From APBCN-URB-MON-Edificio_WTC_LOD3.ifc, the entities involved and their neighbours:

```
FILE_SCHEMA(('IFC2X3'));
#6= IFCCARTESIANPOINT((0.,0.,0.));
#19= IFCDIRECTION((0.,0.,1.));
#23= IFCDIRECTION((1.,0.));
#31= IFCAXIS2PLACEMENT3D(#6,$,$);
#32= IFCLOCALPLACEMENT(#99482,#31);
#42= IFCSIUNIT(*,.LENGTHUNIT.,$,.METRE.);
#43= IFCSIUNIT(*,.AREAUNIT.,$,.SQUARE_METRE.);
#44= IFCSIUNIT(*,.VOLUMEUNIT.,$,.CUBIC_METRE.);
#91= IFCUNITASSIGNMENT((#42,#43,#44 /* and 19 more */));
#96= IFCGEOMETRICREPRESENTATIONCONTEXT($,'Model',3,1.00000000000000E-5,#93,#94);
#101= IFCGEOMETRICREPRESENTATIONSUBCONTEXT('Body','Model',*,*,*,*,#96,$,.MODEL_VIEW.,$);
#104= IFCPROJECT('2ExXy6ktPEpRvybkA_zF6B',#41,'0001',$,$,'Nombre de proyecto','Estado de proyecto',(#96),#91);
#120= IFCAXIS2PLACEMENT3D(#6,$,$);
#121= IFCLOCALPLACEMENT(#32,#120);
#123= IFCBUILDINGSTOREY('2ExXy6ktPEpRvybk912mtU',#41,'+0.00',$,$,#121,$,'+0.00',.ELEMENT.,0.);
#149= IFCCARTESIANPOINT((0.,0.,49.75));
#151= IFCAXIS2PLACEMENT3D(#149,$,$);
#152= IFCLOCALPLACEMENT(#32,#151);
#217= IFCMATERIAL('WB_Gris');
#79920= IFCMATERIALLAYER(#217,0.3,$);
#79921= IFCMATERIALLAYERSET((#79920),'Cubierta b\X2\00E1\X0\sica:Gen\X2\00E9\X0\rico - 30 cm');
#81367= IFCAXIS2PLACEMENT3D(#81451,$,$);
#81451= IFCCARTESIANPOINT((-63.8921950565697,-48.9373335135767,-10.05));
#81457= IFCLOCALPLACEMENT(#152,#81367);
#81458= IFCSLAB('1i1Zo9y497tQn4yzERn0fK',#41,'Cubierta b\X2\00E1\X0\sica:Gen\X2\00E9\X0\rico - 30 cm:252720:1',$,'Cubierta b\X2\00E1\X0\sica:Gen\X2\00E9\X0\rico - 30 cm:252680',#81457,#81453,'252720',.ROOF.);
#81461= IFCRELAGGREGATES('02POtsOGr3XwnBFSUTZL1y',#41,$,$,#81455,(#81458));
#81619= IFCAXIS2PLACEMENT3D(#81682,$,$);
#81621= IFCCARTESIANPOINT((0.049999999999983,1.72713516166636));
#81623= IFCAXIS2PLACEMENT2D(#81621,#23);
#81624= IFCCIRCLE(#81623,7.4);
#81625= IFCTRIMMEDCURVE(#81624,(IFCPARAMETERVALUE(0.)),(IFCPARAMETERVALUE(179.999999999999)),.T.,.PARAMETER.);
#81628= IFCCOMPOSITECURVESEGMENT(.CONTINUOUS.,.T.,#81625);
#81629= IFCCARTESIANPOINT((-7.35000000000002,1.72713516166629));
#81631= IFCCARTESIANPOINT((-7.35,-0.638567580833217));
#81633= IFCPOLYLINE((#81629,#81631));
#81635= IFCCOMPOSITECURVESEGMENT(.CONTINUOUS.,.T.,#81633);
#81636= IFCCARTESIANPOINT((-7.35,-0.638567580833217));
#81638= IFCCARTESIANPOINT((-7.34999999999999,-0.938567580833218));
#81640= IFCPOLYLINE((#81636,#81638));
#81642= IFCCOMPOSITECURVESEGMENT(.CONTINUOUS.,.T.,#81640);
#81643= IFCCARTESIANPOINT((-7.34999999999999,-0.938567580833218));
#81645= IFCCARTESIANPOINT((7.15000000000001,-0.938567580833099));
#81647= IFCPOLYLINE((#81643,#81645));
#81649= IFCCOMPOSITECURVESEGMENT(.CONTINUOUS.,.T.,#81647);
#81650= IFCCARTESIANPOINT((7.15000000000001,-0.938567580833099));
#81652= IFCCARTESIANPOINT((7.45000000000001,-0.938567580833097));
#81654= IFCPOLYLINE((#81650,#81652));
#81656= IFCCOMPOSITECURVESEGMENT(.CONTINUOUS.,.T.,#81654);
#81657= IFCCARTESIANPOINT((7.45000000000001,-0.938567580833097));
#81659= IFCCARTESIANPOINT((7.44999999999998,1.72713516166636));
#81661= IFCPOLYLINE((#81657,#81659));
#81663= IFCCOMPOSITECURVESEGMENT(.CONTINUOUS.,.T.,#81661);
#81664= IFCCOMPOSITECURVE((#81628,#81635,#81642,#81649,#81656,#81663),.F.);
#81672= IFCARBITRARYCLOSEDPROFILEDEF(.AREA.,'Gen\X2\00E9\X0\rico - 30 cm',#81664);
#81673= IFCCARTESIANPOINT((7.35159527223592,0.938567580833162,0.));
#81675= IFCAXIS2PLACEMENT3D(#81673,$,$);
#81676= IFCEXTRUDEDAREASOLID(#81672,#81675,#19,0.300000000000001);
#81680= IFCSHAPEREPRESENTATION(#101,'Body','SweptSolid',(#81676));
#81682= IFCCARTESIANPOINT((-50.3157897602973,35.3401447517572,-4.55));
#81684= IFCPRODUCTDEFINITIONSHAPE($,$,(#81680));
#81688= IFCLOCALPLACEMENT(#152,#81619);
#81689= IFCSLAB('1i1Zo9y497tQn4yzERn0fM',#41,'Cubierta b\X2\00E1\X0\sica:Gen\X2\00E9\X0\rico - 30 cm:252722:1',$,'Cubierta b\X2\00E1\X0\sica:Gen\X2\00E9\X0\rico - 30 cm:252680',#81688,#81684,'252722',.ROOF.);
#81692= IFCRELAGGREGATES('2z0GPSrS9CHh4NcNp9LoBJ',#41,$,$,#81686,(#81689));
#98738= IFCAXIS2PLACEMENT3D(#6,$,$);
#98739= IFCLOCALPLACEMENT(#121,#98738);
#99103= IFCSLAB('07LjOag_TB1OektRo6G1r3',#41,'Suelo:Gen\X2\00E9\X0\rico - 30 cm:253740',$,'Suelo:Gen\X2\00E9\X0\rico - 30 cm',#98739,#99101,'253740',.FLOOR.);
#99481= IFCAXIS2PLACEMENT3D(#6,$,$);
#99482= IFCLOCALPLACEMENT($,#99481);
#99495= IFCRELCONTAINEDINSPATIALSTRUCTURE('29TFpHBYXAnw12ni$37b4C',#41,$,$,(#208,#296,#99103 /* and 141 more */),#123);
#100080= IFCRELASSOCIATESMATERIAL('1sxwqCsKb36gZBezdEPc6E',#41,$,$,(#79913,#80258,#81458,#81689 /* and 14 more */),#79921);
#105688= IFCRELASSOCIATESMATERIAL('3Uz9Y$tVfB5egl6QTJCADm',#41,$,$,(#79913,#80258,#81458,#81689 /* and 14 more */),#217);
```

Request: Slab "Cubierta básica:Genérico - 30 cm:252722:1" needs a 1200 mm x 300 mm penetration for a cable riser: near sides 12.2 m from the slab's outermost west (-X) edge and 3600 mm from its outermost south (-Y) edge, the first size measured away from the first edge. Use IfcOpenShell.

```python
import numpy as np
import ifcopenshell
import ifcopenshell.api.feature
import ifcopenshell.api.geometry
import ifcopenshell.api.root
import ifcopenshell.geom
import ifcopenshell.util.placement
import ifcopenshell.util.representation
import ifcopenshell.util.shape
import ifcopenshell.util.unit

model = ifcopenshell.open("APBCN-URB-MON-Edificio_WTC_LOD3.ifc")
unit_scale = ifcopenshell.util.unit.calculate_unit_scale(model)
settings = ifcopenshell.geom.settings()


def volume(element):
    """Net volume in cubic metres, openings subtracted."""
    shape = ifcopenshell.geom.create_shape(settings, element)
    return ifcopenshell.util.shape.get_volume(shape.geometry)


slab = model.by_id(81689)
before = volume(slab)

# Extent in the slab's own axes, in metres. The edges named are its -X and -Y sides.
slab_shape = ifcopenshell.geom.create_shape(settings, slab)
vertices = ifcopenshell.util.shape.get_vertices(slab_shape.geometry)
x_min, y_min, bottom = vertices.min(axis=0)
top = vertices[:, 2].max()

opening = ifcopenshell.api.root.create_entity(model, ifc_class="IfcOpeningElement", name="Cable riser opening")
context = ifcopenshell.util.representation.get_context(model, "Model", "Body", "MODEL_VIEW")
width, depth = 1.2, 0.3
outline = [(0.0, 0.0), (width, 0.0), (width, depth), (0.0, depth), (0.0, 0.0)]
# Overshoot both faces by 50 mm so the cut is clean.
shape = ifcopenshell.api.geometry.add_slab_representation(
    model, context=context, depth=top - bottom + 0.1, polyline=outline
)
ifcopenshell.api.geometry.assign_representation(model, product=opening, representation=shape)

matrix = ifcopenshell.util.placement.get_local_placement(slab.ObjectPlacement)
matrix[:, 3] = matrix @ np.append(np.array([x_min + 12.2, y_min + 3.6, bottom - 0.05]) / unit_scale, 1.0)
ifcopenshell.api.geometry.edit_object_placement(model, product=opening, matrix=matrix, is_si=False)
ifcopenshell.api.feature.add_feature(model, feature=opening, element=slab)

after = volume(slab)

print(f"slab volume {before:.3f} -> {after:.3f} m3")

model.write("APBCN-URB-MON-Edificio_WTC_LOD3_updated.ifc")
```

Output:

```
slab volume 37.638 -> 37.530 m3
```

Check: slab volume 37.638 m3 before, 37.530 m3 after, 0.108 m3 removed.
